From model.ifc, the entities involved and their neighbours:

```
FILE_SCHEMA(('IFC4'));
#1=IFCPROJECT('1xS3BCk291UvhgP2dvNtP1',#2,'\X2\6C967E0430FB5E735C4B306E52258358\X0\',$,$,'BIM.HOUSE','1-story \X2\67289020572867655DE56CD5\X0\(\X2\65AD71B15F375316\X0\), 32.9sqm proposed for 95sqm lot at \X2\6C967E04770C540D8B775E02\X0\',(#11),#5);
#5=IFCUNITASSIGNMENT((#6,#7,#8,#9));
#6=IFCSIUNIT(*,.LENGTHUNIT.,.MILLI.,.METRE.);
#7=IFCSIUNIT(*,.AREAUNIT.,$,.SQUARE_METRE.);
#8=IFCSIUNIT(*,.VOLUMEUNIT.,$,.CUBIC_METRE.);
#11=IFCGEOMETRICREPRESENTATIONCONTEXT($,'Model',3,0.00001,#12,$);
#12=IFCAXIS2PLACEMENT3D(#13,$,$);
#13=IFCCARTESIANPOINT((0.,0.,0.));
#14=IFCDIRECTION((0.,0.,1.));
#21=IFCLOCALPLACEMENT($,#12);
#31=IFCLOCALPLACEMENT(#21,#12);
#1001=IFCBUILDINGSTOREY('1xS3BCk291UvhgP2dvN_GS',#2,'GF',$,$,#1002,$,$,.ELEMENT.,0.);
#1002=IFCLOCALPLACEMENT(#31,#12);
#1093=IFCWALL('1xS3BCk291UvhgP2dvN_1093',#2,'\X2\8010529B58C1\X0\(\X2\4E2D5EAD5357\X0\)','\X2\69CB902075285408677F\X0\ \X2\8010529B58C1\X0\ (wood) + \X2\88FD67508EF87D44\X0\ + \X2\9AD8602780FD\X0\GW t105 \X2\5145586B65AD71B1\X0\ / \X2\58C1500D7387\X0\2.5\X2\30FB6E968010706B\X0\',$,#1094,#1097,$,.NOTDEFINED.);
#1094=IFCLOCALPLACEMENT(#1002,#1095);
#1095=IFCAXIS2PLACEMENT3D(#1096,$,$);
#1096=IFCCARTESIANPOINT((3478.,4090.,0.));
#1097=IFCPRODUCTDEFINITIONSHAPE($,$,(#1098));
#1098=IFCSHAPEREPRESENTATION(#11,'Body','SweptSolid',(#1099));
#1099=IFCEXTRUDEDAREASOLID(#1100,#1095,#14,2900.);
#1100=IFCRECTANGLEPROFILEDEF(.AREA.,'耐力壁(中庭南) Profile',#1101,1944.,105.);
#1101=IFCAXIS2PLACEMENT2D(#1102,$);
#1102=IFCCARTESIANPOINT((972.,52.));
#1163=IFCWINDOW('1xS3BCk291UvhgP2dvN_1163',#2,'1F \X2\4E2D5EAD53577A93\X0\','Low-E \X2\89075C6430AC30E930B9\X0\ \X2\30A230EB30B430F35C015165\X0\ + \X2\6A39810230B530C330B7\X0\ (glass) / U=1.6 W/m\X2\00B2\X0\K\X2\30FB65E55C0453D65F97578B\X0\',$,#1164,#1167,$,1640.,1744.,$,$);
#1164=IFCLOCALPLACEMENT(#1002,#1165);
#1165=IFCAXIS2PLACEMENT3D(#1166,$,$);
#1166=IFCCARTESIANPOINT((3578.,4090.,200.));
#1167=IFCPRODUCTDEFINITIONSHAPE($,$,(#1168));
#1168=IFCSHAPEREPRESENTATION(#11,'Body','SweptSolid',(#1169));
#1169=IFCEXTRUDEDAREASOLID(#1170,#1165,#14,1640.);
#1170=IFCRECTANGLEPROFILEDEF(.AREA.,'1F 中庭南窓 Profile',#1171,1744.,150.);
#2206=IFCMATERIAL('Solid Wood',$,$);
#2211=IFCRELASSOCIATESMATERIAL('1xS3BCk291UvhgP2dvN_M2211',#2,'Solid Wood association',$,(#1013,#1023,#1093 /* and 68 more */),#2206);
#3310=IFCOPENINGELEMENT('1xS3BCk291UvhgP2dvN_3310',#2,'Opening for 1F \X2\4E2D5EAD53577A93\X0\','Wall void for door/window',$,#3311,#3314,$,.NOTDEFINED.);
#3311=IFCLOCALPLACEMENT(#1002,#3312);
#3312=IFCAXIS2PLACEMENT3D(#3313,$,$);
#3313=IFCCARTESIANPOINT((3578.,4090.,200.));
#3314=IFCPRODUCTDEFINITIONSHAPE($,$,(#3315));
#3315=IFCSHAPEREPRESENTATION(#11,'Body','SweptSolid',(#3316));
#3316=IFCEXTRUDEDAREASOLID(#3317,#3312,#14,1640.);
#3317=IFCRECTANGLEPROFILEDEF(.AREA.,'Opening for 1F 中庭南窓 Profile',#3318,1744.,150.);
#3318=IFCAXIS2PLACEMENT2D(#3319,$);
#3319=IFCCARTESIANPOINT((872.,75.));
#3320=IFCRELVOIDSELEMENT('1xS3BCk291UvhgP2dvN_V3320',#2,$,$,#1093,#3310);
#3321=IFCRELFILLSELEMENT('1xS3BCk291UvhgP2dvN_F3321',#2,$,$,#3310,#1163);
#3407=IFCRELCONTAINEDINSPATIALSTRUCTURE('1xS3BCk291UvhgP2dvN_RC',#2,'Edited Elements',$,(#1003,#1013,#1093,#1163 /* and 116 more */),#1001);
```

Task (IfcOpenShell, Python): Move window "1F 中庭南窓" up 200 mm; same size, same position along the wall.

```python
import numpy as np
import ifcopenshell
import ifcopenshell.api.geometry
import ifcopenshell.util.placement
import ifcopenshell.util.unit

model = ifcopenshell.open("model.ifc")
unit_scale = ifcopenshell.util.unit.calculate_unit_scale(model)

window = model.by_id(1163)
opening = window.FillsVoids[0].RelatingOpeningElement
dz = 0.2 / unit_scale

shift = np.array([0.0, 0.0, dz])
# The window is not placed relative to its opening, so move both.
for product in (opening, window):
    matrix = ifcopenshell.util.placement.get_local_placement(product.ObjectPlacement)
    matrix[:3, 3] += shift
    ifcopenshell.api.geometry.edit_object_placement(model, product=product, matrix=matrix, is_si=False)

print(f"moved by {dz * unit_scale:+.3f} m")

model.write("model_updated.ifc")
```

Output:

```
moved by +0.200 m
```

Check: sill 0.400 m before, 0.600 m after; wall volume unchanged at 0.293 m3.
